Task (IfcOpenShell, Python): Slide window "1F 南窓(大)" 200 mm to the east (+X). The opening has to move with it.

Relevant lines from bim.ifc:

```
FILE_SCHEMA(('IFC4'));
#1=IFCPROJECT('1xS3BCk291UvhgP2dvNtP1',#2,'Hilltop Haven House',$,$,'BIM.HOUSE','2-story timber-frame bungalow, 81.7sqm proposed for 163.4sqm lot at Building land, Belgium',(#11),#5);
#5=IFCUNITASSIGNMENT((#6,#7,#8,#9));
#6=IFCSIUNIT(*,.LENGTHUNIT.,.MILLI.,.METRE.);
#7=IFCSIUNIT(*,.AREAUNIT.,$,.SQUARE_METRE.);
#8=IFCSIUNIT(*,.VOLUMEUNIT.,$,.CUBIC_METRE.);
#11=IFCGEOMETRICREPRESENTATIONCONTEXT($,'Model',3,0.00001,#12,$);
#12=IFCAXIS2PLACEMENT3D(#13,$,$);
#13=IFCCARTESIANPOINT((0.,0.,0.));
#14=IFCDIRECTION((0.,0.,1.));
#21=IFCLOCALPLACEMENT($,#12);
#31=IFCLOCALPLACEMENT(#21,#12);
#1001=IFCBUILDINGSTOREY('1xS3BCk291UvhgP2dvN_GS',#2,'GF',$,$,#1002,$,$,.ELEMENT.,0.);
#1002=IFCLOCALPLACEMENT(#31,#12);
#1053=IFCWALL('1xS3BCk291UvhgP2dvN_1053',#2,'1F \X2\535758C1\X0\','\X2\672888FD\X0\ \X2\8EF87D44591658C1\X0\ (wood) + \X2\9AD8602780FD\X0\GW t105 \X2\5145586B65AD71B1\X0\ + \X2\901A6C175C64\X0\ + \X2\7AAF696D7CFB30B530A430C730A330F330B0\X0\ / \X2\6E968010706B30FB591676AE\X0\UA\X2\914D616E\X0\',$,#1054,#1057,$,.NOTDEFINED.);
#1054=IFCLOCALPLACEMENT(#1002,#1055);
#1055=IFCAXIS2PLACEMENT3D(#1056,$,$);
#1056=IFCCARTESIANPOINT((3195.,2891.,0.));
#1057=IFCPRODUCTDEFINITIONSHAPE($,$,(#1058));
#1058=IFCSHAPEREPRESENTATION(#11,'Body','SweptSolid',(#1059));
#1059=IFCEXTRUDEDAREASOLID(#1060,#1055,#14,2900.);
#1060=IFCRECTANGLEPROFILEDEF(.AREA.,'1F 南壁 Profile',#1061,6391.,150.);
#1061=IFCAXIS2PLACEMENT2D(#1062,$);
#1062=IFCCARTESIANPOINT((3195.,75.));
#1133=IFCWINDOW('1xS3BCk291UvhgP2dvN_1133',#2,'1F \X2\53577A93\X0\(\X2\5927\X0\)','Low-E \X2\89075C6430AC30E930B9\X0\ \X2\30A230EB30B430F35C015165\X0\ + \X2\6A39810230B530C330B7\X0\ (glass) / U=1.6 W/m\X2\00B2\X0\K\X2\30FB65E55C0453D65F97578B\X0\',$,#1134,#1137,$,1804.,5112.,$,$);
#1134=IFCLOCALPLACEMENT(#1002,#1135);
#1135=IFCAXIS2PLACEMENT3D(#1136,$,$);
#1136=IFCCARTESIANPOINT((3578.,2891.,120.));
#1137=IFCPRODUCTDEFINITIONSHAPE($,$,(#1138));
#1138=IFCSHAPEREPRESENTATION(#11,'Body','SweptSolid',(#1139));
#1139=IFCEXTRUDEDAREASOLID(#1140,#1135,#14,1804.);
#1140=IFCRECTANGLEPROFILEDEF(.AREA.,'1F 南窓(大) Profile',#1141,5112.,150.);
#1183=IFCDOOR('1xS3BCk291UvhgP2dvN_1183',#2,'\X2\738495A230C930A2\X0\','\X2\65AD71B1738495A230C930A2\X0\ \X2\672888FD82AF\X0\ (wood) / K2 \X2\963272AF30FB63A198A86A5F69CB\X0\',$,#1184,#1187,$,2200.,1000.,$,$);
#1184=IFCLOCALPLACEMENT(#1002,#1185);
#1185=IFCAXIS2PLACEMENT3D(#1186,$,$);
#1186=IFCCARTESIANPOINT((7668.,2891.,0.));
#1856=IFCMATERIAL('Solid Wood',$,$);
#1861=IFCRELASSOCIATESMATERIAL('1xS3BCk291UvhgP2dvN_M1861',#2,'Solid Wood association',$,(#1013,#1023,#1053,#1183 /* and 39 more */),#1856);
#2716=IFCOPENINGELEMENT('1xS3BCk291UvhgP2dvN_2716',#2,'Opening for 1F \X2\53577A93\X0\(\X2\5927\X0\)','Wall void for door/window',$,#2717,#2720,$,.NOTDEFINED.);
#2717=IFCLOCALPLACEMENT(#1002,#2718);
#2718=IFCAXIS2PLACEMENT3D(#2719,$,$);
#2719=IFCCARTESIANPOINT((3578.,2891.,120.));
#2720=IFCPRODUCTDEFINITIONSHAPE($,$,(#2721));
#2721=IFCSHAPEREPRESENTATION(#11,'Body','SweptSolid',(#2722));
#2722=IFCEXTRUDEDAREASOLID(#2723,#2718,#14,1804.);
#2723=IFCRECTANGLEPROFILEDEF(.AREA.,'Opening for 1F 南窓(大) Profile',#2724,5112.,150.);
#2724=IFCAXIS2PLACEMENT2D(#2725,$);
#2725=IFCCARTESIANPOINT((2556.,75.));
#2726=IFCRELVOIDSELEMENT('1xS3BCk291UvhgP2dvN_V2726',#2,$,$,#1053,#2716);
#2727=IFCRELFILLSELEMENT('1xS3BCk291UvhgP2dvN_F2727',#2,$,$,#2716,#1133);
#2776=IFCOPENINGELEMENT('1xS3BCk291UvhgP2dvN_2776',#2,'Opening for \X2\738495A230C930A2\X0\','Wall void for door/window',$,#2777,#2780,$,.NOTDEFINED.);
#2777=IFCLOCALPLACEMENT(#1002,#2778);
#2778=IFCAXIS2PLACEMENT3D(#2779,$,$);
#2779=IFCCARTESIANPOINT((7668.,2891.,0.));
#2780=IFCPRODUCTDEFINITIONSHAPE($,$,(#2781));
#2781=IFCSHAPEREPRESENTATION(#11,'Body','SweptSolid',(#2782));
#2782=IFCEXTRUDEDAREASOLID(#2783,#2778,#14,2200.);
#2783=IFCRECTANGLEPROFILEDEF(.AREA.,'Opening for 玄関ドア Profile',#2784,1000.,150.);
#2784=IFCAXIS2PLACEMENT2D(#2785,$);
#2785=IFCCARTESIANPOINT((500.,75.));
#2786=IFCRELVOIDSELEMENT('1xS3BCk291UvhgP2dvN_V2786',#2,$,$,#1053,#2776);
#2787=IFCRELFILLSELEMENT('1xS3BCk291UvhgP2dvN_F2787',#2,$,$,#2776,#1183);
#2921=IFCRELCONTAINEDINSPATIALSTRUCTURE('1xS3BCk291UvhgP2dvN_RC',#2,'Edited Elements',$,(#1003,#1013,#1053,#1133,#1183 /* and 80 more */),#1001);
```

```python
import ifcopenshell
import ifcopenshell.api.geometry
import ifcopenshell.util.placement

model = ifcopenshell.open("bim.ifc")

window = model.by_id(1133)
opening = window.FillsVoids[0].RelatingOpeningElement
wall = opening.VoidsElements[0].RelatingBuildingElement

wall_matrix = ifcopenshell.util.placement.get_local_placement(wall.ObjectPlacement)
shift = wall_matrix[:3, 0] * 200.0
before = ifcopenshell.util.placement.get_local_placement(window.ObjectPlacement)[:3, 3].copy()

# The window is not placed relative to its opening, so move both.
for product in (opening, window):
    matrix = ifcopenshell.util.placement.get_local_placement(product.ObjectPlacement)
    matrix[:3, 3] += shift
    ifcopenshell.api.geometry.edit_object_placement(model, product=product, matrix=matrix, is_si=False)

after = ifcopenshell.util.placement.get_local_placement(window.ObjectPlacement)[:3, 3]
print("window moved by", (after - before).round(3) + 0.0)

model.write("bim-out.ifc")
```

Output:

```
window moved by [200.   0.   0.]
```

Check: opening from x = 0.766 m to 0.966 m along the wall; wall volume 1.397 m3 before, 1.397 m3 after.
